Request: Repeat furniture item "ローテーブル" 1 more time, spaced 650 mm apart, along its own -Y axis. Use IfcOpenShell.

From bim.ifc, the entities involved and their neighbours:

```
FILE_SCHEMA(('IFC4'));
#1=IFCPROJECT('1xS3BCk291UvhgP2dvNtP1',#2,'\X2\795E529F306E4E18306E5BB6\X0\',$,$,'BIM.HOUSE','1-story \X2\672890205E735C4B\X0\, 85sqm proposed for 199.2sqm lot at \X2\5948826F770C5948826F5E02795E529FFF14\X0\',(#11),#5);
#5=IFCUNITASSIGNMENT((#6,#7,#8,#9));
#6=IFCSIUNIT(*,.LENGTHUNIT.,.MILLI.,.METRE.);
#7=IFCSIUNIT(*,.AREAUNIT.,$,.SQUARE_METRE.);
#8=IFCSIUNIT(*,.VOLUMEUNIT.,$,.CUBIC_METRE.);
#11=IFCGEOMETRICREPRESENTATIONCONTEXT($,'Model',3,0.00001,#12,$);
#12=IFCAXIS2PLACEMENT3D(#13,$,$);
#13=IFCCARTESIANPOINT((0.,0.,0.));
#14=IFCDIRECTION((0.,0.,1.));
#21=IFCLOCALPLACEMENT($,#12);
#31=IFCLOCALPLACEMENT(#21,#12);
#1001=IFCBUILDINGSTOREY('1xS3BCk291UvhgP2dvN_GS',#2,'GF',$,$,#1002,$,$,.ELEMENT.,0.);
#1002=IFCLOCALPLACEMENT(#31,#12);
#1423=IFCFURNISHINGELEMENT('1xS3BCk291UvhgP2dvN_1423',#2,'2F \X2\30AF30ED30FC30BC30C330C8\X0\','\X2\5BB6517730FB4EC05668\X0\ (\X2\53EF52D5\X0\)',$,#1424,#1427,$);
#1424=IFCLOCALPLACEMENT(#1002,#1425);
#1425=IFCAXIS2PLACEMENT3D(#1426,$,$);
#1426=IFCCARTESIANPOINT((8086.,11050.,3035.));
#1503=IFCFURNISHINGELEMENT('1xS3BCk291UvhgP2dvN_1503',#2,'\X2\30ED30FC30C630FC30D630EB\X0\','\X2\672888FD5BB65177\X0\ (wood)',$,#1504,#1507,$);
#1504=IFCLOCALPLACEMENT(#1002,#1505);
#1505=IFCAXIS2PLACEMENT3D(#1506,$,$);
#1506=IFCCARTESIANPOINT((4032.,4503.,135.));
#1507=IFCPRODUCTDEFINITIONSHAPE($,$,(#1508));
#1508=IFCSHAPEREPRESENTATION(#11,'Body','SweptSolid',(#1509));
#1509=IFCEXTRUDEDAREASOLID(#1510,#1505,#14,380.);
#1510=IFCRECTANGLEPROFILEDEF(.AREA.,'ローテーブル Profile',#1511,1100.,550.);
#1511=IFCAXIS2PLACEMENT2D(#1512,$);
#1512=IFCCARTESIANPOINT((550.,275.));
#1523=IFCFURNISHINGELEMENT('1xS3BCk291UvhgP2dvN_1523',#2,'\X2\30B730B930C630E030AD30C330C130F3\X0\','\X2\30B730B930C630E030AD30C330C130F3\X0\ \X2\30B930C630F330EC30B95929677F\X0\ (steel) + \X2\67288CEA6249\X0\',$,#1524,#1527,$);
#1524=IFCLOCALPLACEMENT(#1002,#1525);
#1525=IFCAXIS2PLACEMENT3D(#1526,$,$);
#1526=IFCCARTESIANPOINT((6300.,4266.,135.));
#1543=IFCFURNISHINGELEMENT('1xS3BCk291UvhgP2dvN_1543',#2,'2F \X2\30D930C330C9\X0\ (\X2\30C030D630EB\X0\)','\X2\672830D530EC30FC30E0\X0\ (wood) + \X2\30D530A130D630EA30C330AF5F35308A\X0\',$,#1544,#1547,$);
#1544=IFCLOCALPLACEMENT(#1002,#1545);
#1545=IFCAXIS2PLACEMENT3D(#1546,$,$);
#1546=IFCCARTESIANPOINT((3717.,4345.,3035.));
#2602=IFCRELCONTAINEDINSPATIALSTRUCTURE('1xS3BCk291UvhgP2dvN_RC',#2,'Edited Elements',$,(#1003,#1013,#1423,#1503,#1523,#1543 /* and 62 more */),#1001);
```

```python
import ifcopenshell
import ifcopenshell.api.geometry
import ifcopenshell.api.root
import ifcopenshell.util.element
import ifcopenshell.util.placement
import ifcopenshell.util.unit

model = ifcopenshell.open("bim.ifc")
unit_scale = ifcopenshell.util.unit.calculate_unit_scale(model)


def reuse_history(source, copy):
    """copy_class also copies each property set's owner history, people and application; keep the originals."""
    for rel in copy.IsDefinedBy:
        if rel.is_a("IfcRelDefinesByProperties") and (history := rel.RelatingPropertyDefinition.OwnerHistory):
            rel.RelatingPropertyDefinition.OwnerHistory = source.OwnerHistory
            ifcopenshell.util.element.remove_deep2(model, history)


source = model.by_id(1503)
base = ifcopenshell.util.placement.get_local_placement(source.ObjectPlacement)
step = -base[:3, 1] * 0.65 / unit_scale

for i in range(1, 2):
    copy = ifcopenshell.api.root.copy_class(model, product=source)
    copy.Representation = ifcopenshell.util.element.copy_deep(
        model, source.Representation, exclude=["IfcGeometricRepresentationContext", "IfcRepresentationMap"]
    )
    reuse_history(source, copy)
    matrix = base.copy()
    matrix[:3, 3] += i * step
    print("added at", matrix[:3, 3].round(3) + 0.0)
    ifcopenshell.api.geometry.edit_object_placement(model, product=copy, matrix=matrix, is_si=False)

model.write("bim_updated.ifc")
```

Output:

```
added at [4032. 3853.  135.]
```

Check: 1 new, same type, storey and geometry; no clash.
